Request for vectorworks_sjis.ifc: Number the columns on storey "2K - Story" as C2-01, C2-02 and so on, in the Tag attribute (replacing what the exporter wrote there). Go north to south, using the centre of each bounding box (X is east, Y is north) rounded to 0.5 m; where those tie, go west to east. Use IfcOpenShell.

First a look at what the model holds.

```python
import ifcopenshell
import ifcopenshell.util.element
import ifcopenshell.util.placement

model = ifcopenshell.open("vectorworks_sjis.ifc")
print(model.schema)
storey = next(s for s in model.by_type("IfcBuildingStorey") if s.Name == '2\x8aK - Story')
columns = [e for e in ifcopenshell.util.element.get_decomposition(storey) if e.is_a("IfcColumn")]
for e in sorted(columns, key=lambda e: e.id()):
    origin = ifcopenshell.util.placement.get_local_placement(e.ObjectPlacement)[:3, 3]
    print(e.id(), e.Tag, e.Name, origin.round(2) + 0.0, sep=" | ")
```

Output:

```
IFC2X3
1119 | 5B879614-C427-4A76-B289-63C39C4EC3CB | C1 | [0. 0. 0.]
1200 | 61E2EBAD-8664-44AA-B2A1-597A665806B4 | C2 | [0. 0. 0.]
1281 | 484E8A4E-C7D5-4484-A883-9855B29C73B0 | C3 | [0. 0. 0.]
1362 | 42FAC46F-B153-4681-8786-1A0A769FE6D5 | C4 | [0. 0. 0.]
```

```python
import ifcopenshell
import ifcopenshell.geom
import ifcopenshell.util.element
import ifcopenshell.util.shape

model = ifcopenshell.open("vectorworks_sjis.ifc")
settings = ifcopenshell.geom.settings()
settings.set("use-world-coords", True)


def centre(element):
    shape = ifcopenshell.geom.create_shape(settings, element)
    return ifcopenshell.util.shape.get_bbox_centroid(shape.geometry)


storey = next(s for s in model.by_type("IfcBuildingStorey") if s.Name == '2\x8aK - Story')
columns = [e for e in ifcopenshell.util.element.get_decomposition(storey) if e.is_a("IfcColumn")]

# Insertion points can sit at a corner or the storey origin, so sort by the geometry (in metres).
centres = {e: centre(e) for e in columns}
columns.sort(key=lambda e: (-round(centres[e][1] / 0.5), centres[e][0]))

for i, e in enumerate(columns, start=1):
    number = f"C2-{i:02d}"
    e.Tag = number
    print(e.id(), number)

model.write("vectorworks_sjis_rev.ifc")
```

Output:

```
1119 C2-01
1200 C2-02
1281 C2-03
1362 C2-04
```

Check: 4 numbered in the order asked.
